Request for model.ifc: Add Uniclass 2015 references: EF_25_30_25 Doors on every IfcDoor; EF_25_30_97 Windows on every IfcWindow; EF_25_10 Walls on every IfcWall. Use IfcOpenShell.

First a look at what the model holds.

```python
import ifcopenshell

model = ifcopenshell.open("model.ifc")
print(model.schema)
print("classifications:", [c.Name for c in model.by_type("IfcClassification")])
for ifc_class in ("IfcDoor", "IfcRoof", "IfcStair", "IfcWall", "IfcWindow"):
    print(ifc_class, len(model.by_type(ifc_class)))
```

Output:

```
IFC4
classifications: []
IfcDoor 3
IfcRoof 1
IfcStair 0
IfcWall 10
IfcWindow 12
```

```python
import ifcopenshell
import ifcopenshell.api.classification

model = ifcopenshell.open("model.ifc")

system = ifcopenshell.api.classification.add_classification(model, classification="Uniclass 2015")

codes = {
    "IfcDoor": ("EF_25_30_25", "Doors"),
    "IfcWindow": ("EF_25_30_97", "Windows"),
    "IfcWall": ("EF_25_10", "Walls"),
}
for ifc_class, (code, name) in codes.items():
    products = model.by_type(ifc_class)
    ifcopenshell.api.classification.add_reference(
        model, products=products, classification=system, identification=code, name=name
    )
    print(code, len(products))

model.write("model_updated.ifc")
```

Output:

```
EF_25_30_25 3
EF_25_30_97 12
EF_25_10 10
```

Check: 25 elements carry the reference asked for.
